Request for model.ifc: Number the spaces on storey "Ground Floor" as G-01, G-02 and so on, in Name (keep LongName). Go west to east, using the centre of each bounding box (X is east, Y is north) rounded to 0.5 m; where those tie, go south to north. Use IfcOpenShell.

First a look at what the model holds.

```python
import ifcopenshell
import ifcopenshell.util.element
import ifcopenshell.util.placement

model = ifcopenshell.open("model.ifc")
print(model.schema)
storey = next(s for s in model.by_type("IfcBuildingStorey") if s.Name == "Ground Floor")
spaces = [e for e in ifcopenshell.util.element.get_decomposition(storey) if e.is_a("IfcSpace")]
for e in sorted(spaces, key=lambda e: e.id()):
    origin = ifcopenshell.util.placement.get_local_placement(e.ObjectPlacement)[:3, 3]
    print(e.id(), e.Name, e.LongName, origin.round(2) + 0.0, sep=" | ")
```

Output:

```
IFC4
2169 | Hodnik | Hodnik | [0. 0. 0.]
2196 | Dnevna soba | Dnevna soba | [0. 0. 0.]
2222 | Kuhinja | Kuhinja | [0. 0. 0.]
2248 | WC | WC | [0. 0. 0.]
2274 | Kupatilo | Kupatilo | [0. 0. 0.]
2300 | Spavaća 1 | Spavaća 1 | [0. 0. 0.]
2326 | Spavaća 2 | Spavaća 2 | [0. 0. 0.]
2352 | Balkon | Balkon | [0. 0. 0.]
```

```python
import ifcopenshell
import ifcopenshell.geom
import ifcopenshell.util.element
import ifcopenshell.util.shape

model = ifcopenshell.open("model.ifc")
settings = ifcopenshell.geom.settings()
settings.set("use-world-coords", True)


def centre(element):
    shape = ifcopenshell.geom.create_shape(settings, element)
    return ifcopenshell.util.shape.get_bbox_centroid(shape.geometry)


storey = next(s for s in model.by_type("IfcBuildingStorey") if s.Name == "Ground Floor")
spaces = [e for e in ifcopenshell.util.element.get_decomposition(storey) if e.is_a("IfcSpace")]

# Insertion points can sit at a corner or the storey origin, so sort by the geometry (in metres).
centres = {e: centre(e) for e in spaces}
spaces.sort(key=lambda e: (round(centres[e][0] / 0.5), centres[e][1]))

for i, e in enumerate(spaces, start=1):
    number = f"G-{i:02d}"
    e.Name = number
    print(e.id(), number)

model.write("model_v2.ifc")
```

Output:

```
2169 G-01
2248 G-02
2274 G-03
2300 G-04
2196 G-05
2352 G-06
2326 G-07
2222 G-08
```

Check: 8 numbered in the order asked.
